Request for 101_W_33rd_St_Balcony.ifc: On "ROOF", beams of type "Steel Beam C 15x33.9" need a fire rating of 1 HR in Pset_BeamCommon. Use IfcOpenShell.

First a look at what the model holds.

```python
import ifcopenshell
import ifcopenshell.util.element

model = ifcopenshell.open("101_W_33rd_St_Balcony.ifc")
print(model.schema)
storey = next(s for s in model.by_type("IfcBuildingStorey") if s.Name == "ROOF")
beams = [e for e in ifcopenshell.util.element.get_decomposition(storey) if e.is_a("IfcBeam")]
seen = {}
for e in beams:
    element_type = ifcopenshell.util.element.get_type(e)
    key = (element_type.Name if element_type != e and element_type else None, ifcopenshell.util.element.get_pset(e, "Pset_BeamCommon", "FireRating"))
    seen[key] = seen.get(key, 0) + 1
for (name, value), count in sorted(seen.items(), key=str):
    print(count, "x", name, "|", value)
```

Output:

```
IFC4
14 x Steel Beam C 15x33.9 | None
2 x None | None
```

```python
import ifcopenshell
import ifcopenshell.api.pset
import ifcopenshell.util.element

model = ifcopenshell.open("101_W_33rd_St_Balcony.ifc")

storey = next(s for s in model.by_type("IfcBuildingStorey") if s.Name == "ROOF")
beams = [e for e in ifcopenshell.util.element.get_decomposition(storey) if e.is_a("IfcBeam")]

count = 0
for e in beams:
    element_type = ifcopenshell.util.element.get_type(e)
    if element_type in (None, e) or element_type.Name != "Steel Beam C 15x33.9":
        continue
    # add_pset returns the element's existing set when there is one.
    pset = ifcopenshell.api.pset.add_pset(model, product=e, name="Pset_BeamCommon")
    ifcopenshell.api.pset.edit_pset(model, pset=pset, properties={"FireRating": "1 HR"})
    count += 1

print(count, "beams updated")

model.write("101_W_33rd_St_Balcony_rev.ifc")
```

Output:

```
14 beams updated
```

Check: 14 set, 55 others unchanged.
